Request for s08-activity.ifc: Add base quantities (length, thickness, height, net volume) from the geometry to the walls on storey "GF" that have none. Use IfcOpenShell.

First a look at what the model holds.

```python
import ifcopenshell
import ifcopenshell.util.element
import ifcopenshell.util.unit

model = ifcopenshell.open("s08-activity.ifc")
print(model.schema)
for unit_type in ("LENGTHUNIT", "AREAUNIT", "VOLUMEUNIT"):
    print(unit_type, ifcopenshell.util.unit.calculate_unit_scale(model, unit_type))
storey = next(s for s in model.by_type("IfcBuildingStorey") if s.Name == "GF")
walls = [e for e in ifcopenshell.util.element.get_decomposition(storey) if e.is_a("IfcWall")]
for e in sorted(walls, key=lambda e: e.id()):
    print(e.id(), e.is_a(), e.Name, list(ifcopenshell.util.element.get_psets(e, qtos_only=True)), sep=" | ")
```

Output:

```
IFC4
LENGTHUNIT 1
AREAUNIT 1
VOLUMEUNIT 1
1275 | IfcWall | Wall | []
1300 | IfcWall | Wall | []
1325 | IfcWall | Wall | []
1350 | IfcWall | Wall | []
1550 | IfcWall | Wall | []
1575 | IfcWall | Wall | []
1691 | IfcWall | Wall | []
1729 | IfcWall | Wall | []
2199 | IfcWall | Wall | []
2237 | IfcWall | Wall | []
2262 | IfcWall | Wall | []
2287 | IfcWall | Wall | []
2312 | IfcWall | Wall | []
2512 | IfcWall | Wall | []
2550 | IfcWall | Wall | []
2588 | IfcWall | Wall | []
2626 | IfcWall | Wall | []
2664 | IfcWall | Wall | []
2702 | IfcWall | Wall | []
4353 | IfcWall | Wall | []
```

```python
import ifcopenshell
import ifcopenshell.api.pset
import ifcopenshell.geom
import ifcopenshell.util.element
import ifcopenshell.util.shape
import ifcopenshell.util.unit

model = ifcopenshell.open("s08-activity.ifc")
unit_scale = ifcopenshell.util.unit.calculate_unit_scale(model)
volume_scale = ifcopenshell.util.unit.calculate_unit_scale(model, "VOLUMEUNIT")
settings = ifcopenshell.geom.settings()

storey = next(s for s in model.by_type("IfcBuildingStorey") if s.Name == "GF")
walls = [e for e in ifcopenshell.util.element.get_decomposition(storey) if e.is_a("IfcWall")]

for e in sorted(walls, key=lambda e: e.id()):
    if ifcopenshell.util.element.get_psets(e, qtos_only=True, should_inherit=False):
        continue
    # Geometry comes back in metres, in the element's own axes.
    shape = ifcopenshell.geom.create_shape(settings, e)
    values = {
        "Length": ifcopenshell.util.shape.get_x(shape.geometry) / unit_scale,
        "Width": ifcopenshell.util.shape.get_y(shape.geometry) / unit_scale,
        "Height": ifcopenshell.util.shape.get_z(shape.geometry) / unit_scale,
        "NetVolume": ifcopenshell.util.shape.get_volume(shape.geometry) / volume_scale,
    }
    qto = ifcopenshell.api.pset.add_qto(model, product=e, name="Qto_WallBaseQuantities")
    ifcopenshell.api.pset.edit_qto(model, qto=qto, properties=values)
    print(e.id(), {k: round(v, 3) for k, v in values.items()})

model.write("s08-activity_updated.ifc")
```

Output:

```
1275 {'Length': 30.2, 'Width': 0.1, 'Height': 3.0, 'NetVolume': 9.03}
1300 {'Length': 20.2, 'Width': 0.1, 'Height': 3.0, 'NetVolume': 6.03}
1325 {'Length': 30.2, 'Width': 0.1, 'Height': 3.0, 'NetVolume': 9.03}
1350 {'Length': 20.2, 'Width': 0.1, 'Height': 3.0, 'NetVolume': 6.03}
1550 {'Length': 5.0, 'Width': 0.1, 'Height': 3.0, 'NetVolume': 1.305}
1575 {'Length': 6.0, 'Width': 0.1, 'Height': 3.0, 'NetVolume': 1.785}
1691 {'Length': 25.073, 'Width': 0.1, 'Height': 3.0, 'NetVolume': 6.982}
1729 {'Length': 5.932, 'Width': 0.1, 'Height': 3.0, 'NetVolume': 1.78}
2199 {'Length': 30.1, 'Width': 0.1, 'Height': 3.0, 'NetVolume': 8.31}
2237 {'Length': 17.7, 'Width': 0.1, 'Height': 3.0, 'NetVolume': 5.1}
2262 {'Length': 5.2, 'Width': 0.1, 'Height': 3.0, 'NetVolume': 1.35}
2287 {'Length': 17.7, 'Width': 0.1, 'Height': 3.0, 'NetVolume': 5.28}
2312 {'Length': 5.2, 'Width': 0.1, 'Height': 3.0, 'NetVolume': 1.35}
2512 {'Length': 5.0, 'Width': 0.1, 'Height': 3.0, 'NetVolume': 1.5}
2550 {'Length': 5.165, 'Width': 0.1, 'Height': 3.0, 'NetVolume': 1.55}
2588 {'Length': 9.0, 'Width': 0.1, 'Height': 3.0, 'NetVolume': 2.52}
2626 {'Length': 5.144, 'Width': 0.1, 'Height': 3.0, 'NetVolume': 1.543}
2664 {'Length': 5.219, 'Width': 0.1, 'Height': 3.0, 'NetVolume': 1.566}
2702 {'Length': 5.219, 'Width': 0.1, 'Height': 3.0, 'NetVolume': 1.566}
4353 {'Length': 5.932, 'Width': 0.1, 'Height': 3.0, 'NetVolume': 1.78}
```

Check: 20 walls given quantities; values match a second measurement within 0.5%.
